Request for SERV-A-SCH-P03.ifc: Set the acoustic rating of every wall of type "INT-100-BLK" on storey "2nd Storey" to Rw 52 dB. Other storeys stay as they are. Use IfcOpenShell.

First a look at what the model holds.

```python
import ifcopenshell
import ifcopenshell.util.element

model = ifcopenshell.open("SERV-A-SCH-P03.ifc")
print(model.schema)
storey = next(s for s in model.by_type("IfcBuildingStorey") if s.Name == "2nd Storey")
walls = [e for e in ifcopenshell.util.element.get_decomposition(storey) if e.is_a("IfcWall")]
seen = {}
for e in walls:
    element_type = ifcopenshell.util.element.get_type(e)
    key = (element_type.Name if element_type != e and element_type else None, ifcopenshell.util.element.get_pset(e, "Pset_WallCommon", "AcousticRating"))
    seen[key] = seen.get(key, 0) + 1
for (name, value), count in sorted(seen.items(), key=str):
    print(count, "x", name, "|", value)
```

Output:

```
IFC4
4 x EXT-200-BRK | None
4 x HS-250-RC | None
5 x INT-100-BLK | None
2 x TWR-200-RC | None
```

```python
import ifcopenshell
import ifcopenshell.api.pset
import ifcopenshell.util.element

model = ifcopenshell.open("SERV-A-SCH-P03.ifc")

storey = next(s for s in model.by_type("IfcBuildingStorey") if s.Name == "2nd Storey")
walls = [e for e in ifcopenshell.util.element.get_decomposition(storey) if e.is_a("IfcWall")]

count = 0
for e in walls:
    element_type = ifcopenshell.util.element.get_type(e)
    if element_type in (None, e) or element_type.Name != "INT-100-BLK":
        continue
    # add_pset returns the element's existing set when there is one.
    pset = ifcopenshell.api.pset.add_pset(model, product=e, name="Pset_WallCommon")
    ifcopenshell.api.pset.edit_pset(model, pset=pset, properties={"AcousticRating": "Rw 52 dB"})
    count += 1

print(count, "walls updated")

model.write("SERV-A-SCH-P03_edited.ifc")
```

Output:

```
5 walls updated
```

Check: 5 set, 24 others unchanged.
